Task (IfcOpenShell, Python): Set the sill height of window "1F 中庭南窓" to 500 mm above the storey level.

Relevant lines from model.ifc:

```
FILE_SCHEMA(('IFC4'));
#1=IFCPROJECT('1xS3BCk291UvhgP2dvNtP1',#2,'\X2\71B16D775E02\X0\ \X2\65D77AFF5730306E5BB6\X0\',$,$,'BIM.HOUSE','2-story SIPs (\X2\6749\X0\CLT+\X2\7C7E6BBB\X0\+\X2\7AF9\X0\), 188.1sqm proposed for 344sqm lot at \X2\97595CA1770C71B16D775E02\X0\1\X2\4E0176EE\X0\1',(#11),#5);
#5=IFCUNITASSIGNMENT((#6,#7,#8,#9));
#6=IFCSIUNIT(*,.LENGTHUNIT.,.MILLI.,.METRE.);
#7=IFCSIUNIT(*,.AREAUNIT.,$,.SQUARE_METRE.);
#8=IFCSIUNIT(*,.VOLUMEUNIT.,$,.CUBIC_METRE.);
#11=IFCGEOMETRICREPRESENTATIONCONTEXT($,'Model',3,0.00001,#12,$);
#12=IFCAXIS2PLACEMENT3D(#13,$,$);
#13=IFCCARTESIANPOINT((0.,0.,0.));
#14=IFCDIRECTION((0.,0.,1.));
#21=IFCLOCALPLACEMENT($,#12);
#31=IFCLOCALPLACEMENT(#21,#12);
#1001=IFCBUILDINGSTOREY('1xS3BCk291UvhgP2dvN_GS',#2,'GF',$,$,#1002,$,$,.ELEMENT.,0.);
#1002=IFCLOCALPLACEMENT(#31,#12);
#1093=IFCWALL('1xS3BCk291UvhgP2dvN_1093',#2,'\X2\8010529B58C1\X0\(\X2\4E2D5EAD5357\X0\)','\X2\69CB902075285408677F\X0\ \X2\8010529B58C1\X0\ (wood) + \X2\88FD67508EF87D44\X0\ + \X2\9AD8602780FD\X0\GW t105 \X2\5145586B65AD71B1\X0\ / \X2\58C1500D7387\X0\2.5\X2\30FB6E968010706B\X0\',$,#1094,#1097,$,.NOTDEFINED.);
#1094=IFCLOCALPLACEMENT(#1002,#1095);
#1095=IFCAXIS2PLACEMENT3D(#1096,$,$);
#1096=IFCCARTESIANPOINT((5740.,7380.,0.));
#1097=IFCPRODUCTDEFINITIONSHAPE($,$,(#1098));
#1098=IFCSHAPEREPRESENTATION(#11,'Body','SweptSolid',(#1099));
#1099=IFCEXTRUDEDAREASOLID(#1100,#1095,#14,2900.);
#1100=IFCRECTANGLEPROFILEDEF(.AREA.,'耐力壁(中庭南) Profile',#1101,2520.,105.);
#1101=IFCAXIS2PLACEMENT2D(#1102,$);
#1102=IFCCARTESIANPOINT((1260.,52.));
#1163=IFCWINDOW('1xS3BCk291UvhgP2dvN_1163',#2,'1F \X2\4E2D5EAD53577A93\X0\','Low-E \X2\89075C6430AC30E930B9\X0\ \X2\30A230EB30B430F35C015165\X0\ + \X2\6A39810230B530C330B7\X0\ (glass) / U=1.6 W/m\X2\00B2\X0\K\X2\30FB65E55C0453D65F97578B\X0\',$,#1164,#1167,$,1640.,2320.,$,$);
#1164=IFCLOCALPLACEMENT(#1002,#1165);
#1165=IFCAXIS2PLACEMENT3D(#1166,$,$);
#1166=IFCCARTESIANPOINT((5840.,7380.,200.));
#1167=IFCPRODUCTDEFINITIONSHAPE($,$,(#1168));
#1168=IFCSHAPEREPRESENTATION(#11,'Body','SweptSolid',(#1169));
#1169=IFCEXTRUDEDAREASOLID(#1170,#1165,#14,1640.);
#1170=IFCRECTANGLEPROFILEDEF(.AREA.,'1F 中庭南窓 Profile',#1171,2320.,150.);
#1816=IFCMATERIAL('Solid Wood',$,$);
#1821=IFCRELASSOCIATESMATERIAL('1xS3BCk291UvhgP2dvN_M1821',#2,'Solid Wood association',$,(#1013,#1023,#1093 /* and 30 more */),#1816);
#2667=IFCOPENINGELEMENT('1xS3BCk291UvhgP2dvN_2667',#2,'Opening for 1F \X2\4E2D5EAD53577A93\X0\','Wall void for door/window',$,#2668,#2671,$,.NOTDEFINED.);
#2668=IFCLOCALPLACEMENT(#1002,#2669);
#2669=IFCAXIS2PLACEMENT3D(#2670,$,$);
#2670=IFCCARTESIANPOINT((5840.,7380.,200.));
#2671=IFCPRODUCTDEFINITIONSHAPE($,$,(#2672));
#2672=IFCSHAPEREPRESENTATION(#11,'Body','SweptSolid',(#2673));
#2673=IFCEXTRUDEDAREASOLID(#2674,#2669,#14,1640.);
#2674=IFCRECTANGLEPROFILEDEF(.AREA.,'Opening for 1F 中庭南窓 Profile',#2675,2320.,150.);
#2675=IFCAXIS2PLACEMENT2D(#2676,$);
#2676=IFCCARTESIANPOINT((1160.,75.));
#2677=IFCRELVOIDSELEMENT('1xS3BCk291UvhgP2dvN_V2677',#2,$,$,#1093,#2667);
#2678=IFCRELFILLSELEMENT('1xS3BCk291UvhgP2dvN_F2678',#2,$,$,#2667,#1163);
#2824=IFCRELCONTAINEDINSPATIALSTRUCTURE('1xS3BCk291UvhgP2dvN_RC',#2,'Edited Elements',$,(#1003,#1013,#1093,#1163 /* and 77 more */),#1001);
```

```python
import numpy as np
import ifcopenshell
import ifcopenshell.api.geometry
import ifcopenshell.geom
import ifcopenshell.util.element
import ifcopenshell.util.placement
import ifcopenshell.util.shape
import ifcopenshell.util.unit

model = ifcopenshell.open("model.ifc")
unit_scale = ifcopenshell.util.unit.calculate_unit_scale(model)

window = model.by_guid("1xS3BCk291UvhgP2dvN_1163")
opening = window.FillsVoids[0].RelatingOpeningElement
storey = ifcopenshell.util.element.get_container(window, ifc_class="IfcBuildingStorey")
level = ifcopenshell.util.placement.get_local_placement(storey.ObjectPlacement)[2, 3]

# The opening's origin need not be at the sill, so measure its lowest point.
shape = ifcopenshell.geom.create_shape(ifcopenshell.geom.settings(), opening)
bottom = ifcopenshell.util.shape.get_shape_bottom_elevation(shape, shape.geometry) / unit_scale
dz = level + 500.0 - bottom

shift = np.array([0.0, 0.0, dz])
# The window is not placed relative to its opening, so move both.
for product in (opening, window):
    matrix = ifcopenshell.util.placement.get_local_placement(product.ObjectPlacement)
    matrix[:3, 3] += shift
    ifcopenshell.api.geometry.edit_object_placement(model, product=product, matrix=matrix, is_si=False)

print(f"moved by {dz * unit_scale:+.3f} m")

model.write("model_updated.ifc")
```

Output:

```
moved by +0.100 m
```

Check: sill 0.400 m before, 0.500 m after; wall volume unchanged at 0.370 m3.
